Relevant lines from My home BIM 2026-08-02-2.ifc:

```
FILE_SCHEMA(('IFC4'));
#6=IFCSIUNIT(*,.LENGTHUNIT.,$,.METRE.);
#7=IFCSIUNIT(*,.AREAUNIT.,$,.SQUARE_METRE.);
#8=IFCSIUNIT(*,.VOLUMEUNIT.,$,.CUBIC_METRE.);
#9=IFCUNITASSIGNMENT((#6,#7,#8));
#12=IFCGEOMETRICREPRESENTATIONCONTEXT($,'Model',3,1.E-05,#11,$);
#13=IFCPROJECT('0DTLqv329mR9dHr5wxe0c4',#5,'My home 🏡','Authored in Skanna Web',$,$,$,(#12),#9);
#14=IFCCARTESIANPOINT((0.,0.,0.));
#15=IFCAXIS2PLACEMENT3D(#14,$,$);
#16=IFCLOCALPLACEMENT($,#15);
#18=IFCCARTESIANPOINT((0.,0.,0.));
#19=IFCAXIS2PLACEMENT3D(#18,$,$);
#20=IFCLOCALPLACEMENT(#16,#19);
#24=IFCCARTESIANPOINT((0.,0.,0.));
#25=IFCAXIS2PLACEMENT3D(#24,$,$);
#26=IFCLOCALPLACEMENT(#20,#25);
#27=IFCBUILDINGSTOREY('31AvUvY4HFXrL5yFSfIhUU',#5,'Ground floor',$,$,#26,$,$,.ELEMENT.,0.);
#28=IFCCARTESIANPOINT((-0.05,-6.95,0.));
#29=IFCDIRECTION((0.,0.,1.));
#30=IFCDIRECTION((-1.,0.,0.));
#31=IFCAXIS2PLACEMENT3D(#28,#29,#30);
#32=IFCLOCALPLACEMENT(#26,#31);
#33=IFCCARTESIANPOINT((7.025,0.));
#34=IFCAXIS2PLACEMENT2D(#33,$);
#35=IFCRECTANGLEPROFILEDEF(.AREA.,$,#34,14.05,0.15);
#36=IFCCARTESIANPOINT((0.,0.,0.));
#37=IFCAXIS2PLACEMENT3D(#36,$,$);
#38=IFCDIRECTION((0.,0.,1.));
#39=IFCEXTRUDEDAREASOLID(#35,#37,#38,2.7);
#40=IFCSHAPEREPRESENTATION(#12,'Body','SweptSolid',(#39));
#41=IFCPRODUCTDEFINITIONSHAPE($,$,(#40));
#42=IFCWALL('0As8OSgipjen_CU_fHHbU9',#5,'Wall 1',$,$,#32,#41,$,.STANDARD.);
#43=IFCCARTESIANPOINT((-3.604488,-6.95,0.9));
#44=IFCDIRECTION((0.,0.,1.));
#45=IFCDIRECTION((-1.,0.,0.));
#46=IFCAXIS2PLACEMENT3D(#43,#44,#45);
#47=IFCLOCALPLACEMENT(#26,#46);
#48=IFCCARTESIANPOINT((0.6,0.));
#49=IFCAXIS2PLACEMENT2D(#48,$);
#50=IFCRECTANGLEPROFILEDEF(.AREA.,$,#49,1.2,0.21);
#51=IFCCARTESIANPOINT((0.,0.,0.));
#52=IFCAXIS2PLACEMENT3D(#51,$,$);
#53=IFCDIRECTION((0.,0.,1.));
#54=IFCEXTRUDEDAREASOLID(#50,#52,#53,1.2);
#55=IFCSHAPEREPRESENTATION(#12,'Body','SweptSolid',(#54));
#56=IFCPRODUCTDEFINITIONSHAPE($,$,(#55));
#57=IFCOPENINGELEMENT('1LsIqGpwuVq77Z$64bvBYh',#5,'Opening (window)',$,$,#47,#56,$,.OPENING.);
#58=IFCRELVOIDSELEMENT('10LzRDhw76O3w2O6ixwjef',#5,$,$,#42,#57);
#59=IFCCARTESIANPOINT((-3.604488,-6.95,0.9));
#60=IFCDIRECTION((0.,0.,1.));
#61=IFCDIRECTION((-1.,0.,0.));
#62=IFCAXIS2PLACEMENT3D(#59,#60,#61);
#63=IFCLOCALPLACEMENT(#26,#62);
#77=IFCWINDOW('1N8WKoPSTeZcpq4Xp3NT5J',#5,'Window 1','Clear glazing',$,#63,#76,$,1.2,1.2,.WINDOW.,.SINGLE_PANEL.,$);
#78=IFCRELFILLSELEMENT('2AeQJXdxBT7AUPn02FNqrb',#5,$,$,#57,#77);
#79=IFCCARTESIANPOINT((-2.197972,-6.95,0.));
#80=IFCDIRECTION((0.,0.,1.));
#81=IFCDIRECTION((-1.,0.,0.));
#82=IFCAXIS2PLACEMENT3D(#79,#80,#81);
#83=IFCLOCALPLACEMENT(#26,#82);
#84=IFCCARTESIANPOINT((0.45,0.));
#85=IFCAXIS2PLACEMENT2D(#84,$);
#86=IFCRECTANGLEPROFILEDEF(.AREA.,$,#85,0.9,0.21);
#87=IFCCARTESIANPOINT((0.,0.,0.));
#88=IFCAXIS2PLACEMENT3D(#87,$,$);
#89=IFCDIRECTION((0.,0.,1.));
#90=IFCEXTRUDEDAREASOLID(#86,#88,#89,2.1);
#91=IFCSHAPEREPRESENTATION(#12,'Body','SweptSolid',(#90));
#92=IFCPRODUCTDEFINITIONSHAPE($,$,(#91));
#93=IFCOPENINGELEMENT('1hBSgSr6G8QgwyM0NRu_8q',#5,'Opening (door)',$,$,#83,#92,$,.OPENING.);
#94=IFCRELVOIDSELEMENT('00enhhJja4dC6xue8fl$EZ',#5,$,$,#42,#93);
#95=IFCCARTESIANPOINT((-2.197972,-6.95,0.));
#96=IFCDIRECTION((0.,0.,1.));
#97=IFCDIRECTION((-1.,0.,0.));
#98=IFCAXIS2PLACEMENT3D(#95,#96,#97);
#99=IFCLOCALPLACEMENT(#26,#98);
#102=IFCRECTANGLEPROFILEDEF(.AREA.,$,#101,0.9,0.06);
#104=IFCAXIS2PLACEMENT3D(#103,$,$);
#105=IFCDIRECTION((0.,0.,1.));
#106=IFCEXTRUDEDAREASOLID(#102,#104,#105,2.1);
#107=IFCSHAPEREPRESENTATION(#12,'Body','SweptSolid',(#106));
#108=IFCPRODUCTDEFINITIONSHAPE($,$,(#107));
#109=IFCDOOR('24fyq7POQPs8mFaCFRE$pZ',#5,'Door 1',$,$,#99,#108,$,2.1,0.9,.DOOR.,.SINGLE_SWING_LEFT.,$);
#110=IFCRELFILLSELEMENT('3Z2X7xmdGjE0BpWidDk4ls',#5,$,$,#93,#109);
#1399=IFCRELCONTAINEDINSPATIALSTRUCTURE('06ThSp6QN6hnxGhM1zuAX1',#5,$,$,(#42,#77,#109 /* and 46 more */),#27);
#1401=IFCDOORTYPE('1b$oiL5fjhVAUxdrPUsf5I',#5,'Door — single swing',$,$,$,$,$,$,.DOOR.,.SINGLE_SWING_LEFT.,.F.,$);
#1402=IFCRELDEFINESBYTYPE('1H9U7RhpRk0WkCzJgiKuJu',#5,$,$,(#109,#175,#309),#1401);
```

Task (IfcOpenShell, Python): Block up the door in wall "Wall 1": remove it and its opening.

```python
import ifcopenshell
import ifcopenshell.api.feature
import ifcopenshell.api.root
import ifcopenshell.geom
import ifcopenshell.util.shape

model = ifcopenshell.open("My home BIM 2026-08-02-2.ifc")
settings = ifcopenshell.geom.settings()


def volume(element):
    """Net volume in cubic metres, openings subtracted."""
    shape = ifcopenshell.geom.create_shape(settings, element)
    return ifcopenshell.util.shape.get_volume(shape.geometry)


door = model.by_id(109)
opening = door.FillsVoids[0].RelatingOpeningElement
wall = opening.VoidsElements[0].RelatingBuildingElement
before = volume(wall)

ifcopenshell.api.root.remove_product(model, product=door)
ifcopenshell.api.feature.remove_feature(model, feature=opening)

after = volume(wall)

print(f"wall volume {before:.3f} -> {after:.3f} m3")

model.write("My home BIM 2026-08-02-2-out.ifc")
```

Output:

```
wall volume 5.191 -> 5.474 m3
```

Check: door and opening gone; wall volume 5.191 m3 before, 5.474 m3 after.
